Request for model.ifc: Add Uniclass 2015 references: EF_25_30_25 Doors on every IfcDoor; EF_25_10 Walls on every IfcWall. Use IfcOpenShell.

First a look at what the model holds.

```python
import ifcopenshell

model = ifcopenshell.open("model.ifc")
print(model.schema)
print("classifications:", [c.Name for c in model.by_type("IfcClassification")])
for ifc_class in ("IfcDoor", "IfcRoof", "IfcStair", "IfcWall", "IfcWindow"):
    print(ifc_class, len(model.by_type(ifc_class)))
```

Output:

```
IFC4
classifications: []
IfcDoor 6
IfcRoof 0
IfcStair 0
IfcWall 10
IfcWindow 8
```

```python
import ifcopenshell
import ifcopenshell.api.classification

model = ifcopenshell.open("model.ifc")

system = ifcopenshell.api.classification.add_classification(model, classification="Uniclass 2015")

codes = {
    "IfcDoor": ("EF_25_30_25", "Doors"),
    "IfcWall": ("EF_25_10", "Walls"),
}
for ifc_class, (code, name) in codes.items():
    products = model.by_type(ifc_class)
    ifcopenshell.api.classification.add_reference(
        model, products=products, classification=system, identification=code, name=name
    )
    print(code, len(products))

model.write("model-out.ifc")
```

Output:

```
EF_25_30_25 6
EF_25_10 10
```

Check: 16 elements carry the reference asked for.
